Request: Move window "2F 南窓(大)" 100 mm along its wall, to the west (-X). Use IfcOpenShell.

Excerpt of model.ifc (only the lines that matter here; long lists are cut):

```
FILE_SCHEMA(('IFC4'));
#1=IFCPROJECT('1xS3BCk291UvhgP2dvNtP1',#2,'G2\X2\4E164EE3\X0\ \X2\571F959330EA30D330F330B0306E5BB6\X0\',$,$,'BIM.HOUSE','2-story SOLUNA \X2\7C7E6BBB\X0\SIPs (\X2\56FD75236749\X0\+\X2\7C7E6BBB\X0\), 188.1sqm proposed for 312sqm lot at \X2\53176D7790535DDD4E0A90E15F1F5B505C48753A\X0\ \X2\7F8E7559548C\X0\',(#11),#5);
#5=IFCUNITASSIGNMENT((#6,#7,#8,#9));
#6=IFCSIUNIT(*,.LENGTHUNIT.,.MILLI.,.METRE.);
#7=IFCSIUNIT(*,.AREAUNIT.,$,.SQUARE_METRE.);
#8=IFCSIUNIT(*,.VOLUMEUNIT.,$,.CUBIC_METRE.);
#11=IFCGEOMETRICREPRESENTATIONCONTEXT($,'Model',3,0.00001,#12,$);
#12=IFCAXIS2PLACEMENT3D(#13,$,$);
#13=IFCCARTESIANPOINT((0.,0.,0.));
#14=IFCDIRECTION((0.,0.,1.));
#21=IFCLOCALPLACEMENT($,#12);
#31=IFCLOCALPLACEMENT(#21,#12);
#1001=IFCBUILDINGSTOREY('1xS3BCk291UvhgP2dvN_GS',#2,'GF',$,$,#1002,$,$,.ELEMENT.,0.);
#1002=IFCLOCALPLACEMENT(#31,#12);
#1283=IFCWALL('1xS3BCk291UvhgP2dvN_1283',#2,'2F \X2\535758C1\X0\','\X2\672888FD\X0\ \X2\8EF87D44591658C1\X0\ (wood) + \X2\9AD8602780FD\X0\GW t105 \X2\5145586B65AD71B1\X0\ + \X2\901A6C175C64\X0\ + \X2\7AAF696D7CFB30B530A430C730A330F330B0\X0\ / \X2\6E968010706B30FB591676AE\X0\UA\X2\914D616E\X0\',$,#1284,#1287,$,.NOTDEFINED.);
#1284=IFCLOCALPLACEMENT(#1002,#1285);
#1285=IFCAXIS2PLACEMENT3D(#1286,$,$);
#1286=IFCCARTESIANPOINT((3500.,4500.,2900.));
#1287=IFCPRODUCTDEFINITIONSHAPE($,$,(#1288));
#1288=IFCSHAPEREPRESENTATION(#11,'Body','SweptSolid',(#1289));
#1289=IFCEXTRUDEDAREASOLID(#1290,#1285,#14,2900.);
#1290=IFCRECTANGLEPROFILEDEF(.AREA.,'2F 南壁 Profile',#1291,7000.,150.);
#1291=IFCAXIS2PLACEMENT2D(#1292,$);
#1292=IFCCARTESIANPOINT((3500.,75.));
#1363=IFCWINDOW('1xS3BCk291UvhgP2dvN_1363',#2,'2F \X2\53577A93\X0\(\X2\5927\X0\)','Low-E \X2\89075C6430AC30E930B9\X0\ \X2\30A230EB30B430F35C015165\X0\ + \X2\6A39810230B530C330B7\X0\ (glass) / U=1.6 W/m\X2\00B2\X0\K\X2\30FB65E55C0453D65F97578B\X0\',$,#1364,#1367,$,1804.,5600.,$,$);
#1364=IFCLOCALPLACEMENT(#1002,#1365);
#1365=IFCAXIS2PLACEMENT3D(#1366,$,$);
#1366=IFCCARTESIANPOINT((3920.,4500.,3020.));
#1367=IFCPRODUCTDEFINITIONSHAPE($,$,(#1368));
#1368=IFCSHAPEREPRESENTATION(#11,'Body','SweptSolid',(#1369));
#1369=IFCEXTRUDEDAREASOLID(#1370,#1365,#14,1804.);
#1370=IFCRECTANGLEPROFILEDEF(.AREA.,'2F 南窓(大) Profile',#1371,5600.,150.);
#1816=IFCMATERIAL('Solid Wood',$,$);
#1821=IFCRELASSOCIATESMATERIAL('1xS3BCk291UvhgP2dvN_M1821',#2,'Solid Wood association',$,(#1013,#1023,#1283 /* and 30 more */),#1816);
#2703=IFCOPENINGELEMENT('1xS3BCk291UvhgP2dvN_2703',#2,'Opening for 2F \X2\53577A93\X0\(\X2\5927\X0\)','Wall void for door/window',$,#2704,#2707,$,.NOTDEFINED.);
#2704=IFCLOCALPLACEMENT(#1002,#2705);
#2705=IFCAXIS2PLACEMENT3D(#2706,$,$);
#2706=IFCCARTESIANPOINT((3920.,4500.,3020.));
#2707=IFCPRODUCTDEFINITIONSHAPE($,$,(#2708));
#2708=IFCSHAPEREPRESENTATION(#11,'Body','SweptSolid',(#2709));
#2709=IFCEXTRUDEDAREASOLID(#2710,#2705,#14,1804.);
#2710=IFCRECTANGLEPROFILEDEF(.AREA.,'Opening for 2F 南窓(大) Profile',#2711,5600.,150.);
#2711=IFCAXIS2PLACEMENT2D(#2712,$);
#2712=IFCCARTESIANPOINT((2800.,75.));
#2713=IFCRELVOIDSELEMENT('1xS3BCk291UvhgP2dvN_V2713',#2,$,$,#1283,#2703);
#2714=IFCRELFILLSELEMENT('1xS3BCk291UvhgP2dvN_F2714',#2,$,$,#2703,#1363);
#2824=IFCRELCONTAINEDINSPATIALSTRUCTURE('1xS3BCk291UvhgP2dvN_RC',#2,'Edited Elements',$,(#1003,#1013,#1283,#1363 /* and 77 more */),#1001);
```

```python
import ifcopenshell
import ifcopenshell.api.geometry
import ifcopenshell.util.placement
import ifcopenshell.util.unit

model = ifcopenshell.open("model.ifc")
unit_scale = ifcopenshell.util.unit.calculate_unit_scale(model)

window = model.by_guid("1xS3BCk291UvhgP2dvN_1363")
opening = window.FillsVoids[0].RelatingOpeningElement
wall = opening.VoidsElements[0].RelatingBuildingElement

wall_matrix = ifcopenshell.util.placement.get_local_placement(wall.ObjectPlacement)
shift = wall_matrix[:3, 0] * -0.1 / unit_scale
before = ifcopenshell.util.placement.get_local_placement(window.ObjectPlacement)[:3, 3].copy()

# The window is not placed relative to its opening, so move both.
for product in (opening, window):
    matrix = ifcopenshell.util.placement.get_local_placement(product.ObjectPlacement)
    matrix[:3, 3] += shift
    ifcopenshell.api.geometry.edit_object_placement(model, product=product, matrix=matrix, is_si=False)

after = ifcopenshell.util.placement.get_local_placement(window.ObjectPlacement)[:3, 3]
print("window moved by", (after - before).round(3) + 0.0)

model.write("model-out.ifc")
```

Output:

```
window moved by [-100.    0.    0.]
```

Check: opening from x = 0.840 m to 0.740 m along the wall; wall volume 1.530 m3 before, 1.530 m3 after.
